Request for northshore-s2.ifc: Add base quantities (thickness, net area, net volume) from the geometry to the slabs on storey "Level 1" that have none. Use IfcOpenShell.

First a look at what the model holds.

```python
import ifcopenshell
import ifcopenshell.util.element
import ifcopenshell.util.unit

model = ifcopenshell.open("northshore-s2.ifc")
print(model.schema)
for unit_type in ("LENGTHUNIT", "AREAUNIT", "VOLUMEUNIT"):
    print(unit_type, ifcopenshell.util.unit.calculate_unit_scale(model, unit_type))
storey = next(s for s in model.by_type("IfcBuildingStorey") if s.Name == "Level 1")
slabs = [e for e in ifcopenshell.util.element.get_decomposition(storey) if e.is_a("IfcSlab")]
for e in sorted(slabs, key=lambda e: e.id()):
    print(e.id(), e.is_a(), e.Name, list(ifcopenshell.util.element.get_psets(e, qtos_only=True)), sep=" | ")
```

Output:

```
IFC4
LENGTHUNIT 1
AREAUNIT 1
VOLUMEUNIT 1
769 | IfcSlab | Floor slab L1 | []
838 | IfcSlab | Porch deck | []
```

```python
import ifcopenshell
import ifcopenshell.api.pset
import ifcopenshell.geom
import ifcopenshell.util.element
import ifcopenshell.util.shape
import ifcopenshell.util.unit

model = ifcopenshell.open("northshore-s2.ifc")
unit_scale = ifcopenshell.util.unit.calculate_unit_scale(model)
area_scale = ifcopenshell.util.unit.calculate_unit_scale(model, "AREAUNIT")
volume_scale = ifcopenshell.util.unit.calculate_unit_scale(model, "VOLUMEUNIT")
settings = ifcopenshell.geom.settings()

storey = next(s for s in model.by_type("IfcBuildingStorey") if s.Name == "Level 1")
slabs = [e for e in ifcopenshell.util.element.get_decomposition(storey) if e.is_a("IfcSlab")]

for e in sorted(slabs, key=lambda e: e.id()):
    if ifcopenshell.util.element.get_psets(e, qtos_only=True, should_inherit=False):
        continue
    # Geometry comes back in metres, in the element's own axes.
    shape = ifcopenshell.geom.create_shape(settings, e)
    values = {
        "Width": ifcopenshell.util.shape.get_z(shape.geometry) / unit_scale,
        "NetArea": ifcopenshell.util.shape.get_footprint_area(shape.geometry) / area_scale,
        "NetVolume": ifcopenshell.util.shape.get_volume(shape.geometry) / volume_scale,
    }
    qto = ifcopenshell.api.pset.add_qto(model, product=e, name="Qto_SlabBaseQuantities")
    ifcopenshell.api.pset.edit_qto(model, qto=qto, properties=values)
    print(e.id(), {k: round(v, 3) for k, v in values.items()})

model.write("northshore-s2_updated.ifc")
```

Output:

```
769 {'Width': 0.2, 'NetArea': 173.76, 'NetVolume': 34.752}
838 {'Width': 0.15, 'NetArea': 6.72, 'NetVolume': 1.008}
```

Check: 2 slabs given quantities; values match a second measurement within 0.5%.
